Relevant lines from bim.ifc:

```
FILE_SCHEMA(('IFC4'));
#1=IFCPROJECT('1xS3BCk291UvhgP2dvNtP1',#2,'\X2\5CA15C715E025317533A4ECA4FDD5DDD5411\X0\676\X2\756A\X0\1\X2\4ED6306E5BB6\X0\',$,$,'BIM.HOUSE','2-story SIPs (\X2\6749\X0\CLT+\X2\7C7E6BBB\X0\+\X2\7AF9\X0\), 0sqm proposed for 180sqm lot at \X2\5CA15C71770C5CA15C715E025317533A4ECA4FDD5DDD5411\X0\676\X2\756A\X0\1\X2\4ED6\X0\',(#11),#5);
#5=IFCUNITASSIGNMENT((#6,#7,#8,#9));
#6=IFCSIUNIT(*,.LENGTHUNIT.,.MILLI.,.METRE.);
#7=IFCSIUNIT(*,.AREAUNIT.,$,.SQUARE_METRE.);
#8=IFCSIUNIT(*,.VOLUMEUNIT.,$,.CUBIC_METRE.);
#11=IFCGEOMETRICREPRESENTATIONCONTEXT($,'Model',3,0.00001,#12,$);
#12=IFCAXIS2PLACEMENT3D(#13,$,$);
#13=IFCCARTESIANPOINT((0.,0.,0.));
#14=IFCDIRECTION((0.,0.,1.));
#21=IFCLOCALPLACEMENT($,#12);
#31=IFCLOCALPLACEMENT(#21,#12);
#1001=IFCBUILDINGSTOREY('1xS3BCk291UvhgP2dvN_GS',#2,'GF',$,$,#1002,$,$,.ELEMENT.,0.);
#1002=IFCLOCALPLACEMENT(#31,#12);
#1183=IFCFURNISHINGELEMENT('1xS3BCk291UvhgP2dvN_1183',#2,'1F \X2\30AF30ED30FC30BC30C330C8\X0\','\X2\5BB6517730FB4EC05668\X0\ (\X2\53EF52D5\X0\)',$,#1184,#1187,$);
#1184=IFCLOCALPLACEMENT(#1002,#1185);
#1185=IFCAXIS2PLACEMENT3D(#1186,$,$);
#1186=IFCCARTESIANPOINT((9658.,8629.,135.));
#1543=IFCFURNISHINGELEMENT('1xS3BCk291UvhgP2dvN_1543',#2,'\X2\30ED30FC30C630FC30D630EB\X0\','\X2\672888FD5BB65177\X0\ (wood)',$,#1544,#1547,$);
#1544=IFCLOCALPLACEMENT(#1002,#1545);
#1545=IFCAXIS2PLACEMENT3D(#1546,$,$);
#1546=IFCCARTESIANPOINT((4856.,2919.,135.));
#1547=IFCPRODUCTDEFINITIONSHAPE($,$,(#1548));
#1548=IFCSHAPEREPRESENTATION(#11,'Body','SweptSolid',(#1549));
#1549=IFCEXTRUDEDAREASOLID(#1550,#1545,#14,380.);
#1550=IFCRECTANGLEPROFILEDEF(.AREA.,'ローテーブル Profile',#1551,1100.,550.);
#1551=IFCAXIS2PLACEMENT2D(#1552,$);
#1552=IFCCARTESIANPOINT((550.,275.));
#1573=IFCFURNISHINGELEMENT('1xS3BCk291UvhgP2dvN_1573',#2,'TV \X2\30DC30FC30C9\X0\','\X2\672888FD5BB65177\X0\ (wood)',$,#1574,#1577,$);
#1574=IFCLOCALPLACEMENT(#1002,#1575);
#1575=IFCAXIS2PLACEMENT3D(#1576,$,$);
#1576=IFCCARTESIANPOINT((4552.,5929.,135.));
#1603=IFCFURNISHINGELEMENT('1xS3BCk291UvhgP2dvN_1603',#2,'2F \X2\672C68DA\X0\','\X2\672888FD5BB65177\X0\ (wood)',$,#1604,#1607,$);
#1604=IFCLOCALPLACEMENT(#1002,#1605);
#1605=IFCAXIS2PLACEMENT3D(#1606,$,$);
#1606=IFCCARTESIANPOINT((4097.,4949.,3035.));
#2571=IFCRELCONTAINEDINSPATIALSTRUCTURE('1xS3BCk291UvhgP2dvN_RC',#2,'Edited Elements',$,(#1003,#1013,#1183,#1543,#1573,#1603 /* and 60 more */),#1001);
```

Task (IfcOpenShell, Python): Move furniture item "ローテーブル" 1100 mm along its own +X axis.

```python
import ifcopenshell
import ifcopenshell.api.geometry
import ifcopenshell.util.placement

model = ifcopenshell.open("bim.ifc")

item = model.by_guid("1xS3BCk291UvhgP2dvN_1543")
matrix = ifcopenshell.util.placement.get_local_placement(item.ObjectPlacement)
matrix[:3, 3] += matrix[:3, 0] * 1100.0
ifcopenshell.api.geometry.edit_object_placement(model, product=item, matrix=matrix, is_si=False)

print(ifcopenshell.util.placement.get_local_placement(item.ObjectPlacement).round(3) + 0.0)

model.write("bim_v2.ifc")
```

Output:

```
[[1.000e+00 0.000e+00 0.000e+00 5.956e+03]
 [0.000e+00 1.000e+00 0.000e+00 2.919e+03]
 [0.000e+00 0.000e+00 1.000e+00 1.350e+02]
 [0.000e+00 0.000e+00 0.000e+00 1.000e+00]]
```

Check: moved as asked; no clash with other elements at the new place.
